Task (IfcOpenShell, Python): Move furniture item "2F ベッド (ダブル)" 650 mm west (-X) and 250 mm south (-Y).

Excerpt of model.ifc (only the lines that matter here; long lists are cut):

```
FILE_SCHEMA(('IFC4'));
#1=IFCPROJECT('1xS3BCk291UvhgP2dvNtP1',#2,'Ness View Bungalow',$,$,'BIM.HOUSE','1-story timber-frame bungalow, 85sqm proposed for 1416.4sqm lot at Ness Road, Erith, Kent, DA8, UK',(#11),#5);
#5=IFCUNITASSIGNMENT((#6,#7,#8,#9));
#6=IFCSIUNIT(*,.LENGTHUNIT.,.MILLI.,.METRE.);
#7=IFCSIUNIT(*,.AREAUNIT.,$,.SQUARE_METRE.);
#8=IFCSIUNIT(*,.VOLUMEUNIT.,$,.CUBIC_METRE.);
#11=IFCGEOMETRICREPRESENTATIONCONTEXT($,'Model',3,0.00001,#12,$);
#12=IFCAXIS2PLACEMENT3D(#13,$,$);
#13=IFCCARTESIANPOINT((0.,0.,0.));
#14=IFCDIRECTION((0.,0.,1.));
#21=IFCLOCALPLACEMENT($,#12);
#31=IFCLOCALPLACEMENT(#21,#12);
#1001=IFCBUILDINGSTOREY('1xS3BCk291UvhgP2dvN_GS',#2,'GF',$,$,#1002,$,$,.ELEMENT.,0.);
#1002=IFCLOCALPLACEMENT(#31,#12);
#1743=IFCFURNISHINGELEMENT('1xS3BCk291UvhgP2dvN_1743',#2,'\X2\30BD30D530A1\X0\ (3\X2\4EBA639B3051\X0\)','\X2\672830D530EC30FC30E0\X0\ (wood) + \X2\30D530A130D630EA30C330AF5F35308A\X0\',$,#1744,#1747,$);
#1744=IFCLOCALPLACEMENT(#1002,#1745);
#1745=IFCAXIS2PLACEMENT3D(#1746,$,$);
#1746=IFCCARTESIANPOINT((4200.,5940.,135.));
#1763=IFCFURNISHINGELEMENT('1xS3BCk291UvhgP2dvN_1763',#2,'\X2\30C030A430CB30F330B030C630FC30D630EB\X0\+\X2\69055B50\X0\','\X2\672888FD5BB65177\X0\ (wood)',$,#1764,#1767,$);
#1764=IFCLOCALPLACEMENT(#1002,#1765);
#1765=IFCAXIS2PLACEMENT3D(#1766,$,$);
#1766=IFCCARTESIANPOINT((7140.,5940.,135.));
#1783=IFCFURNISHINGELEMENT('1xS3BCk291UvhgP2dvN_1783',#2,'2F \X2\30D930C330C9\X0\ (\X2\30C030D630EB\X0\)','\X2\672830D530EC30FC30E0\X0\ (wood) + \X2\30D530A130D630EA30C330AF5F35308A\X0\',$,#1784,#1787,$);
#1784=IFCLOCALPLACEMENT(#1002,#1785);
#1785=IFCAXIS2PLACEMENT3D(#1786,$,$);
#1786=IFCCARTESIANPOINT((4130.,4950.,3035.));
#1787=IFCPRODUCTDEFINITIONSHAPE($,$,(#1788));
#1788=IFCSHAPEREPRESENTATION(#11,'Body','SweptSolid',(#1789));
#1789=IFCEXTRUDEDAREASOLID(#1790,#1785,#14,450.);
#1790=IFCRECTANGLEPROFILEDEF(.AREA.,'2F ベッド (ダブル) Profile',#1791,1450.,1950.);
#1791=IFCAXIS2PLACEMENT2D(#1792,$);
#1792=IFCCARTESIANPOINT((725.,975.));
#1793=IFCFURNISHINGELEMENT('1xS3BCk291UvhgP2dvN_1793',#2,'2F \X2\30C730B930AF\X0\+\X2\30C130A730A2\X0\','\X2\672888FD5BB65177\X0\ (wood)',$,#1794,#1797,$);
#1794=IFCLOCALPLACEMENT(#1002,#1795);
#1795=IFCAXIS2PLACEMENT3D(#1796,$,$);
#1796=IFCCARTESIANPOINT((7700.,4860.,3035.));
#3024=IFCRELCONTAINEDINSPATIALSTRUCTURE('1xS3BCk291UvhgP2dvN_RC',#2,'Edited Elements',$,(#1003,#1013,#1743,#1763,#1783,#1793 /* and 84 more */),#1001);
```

```python
import ifcopenshell
import ifcopenshell.api.geometry
import ifcopenshell.util.placement

model = ifcopenshell.open("model.ifc")

item = model.by_guid("1xS3BCk291UvhgP2dvN_1783")
matrix = ifcopenshell.util.placement.get_local_placement(item.ObjectPlacement)
matrix[0, 3] -= 650.0
matrix[1, 3] -= 250.0
ifcopenshell.api.geometry.edit_object_placement(model, product=item, matrix=matrix, is_si=False)

print(ifcopenshell.util.placement.get_local_placement(item.ObjectPlacement).round(3) + 0.0)

model.write("model_v2.ifc")
```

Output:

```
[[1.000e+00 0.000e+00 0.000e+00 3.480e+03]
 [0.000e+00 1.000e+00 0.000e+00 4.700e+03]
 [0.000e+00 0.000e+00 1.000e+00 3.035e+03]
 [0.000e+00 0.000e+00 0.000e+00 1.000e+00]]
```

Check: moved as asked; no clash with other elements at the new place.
